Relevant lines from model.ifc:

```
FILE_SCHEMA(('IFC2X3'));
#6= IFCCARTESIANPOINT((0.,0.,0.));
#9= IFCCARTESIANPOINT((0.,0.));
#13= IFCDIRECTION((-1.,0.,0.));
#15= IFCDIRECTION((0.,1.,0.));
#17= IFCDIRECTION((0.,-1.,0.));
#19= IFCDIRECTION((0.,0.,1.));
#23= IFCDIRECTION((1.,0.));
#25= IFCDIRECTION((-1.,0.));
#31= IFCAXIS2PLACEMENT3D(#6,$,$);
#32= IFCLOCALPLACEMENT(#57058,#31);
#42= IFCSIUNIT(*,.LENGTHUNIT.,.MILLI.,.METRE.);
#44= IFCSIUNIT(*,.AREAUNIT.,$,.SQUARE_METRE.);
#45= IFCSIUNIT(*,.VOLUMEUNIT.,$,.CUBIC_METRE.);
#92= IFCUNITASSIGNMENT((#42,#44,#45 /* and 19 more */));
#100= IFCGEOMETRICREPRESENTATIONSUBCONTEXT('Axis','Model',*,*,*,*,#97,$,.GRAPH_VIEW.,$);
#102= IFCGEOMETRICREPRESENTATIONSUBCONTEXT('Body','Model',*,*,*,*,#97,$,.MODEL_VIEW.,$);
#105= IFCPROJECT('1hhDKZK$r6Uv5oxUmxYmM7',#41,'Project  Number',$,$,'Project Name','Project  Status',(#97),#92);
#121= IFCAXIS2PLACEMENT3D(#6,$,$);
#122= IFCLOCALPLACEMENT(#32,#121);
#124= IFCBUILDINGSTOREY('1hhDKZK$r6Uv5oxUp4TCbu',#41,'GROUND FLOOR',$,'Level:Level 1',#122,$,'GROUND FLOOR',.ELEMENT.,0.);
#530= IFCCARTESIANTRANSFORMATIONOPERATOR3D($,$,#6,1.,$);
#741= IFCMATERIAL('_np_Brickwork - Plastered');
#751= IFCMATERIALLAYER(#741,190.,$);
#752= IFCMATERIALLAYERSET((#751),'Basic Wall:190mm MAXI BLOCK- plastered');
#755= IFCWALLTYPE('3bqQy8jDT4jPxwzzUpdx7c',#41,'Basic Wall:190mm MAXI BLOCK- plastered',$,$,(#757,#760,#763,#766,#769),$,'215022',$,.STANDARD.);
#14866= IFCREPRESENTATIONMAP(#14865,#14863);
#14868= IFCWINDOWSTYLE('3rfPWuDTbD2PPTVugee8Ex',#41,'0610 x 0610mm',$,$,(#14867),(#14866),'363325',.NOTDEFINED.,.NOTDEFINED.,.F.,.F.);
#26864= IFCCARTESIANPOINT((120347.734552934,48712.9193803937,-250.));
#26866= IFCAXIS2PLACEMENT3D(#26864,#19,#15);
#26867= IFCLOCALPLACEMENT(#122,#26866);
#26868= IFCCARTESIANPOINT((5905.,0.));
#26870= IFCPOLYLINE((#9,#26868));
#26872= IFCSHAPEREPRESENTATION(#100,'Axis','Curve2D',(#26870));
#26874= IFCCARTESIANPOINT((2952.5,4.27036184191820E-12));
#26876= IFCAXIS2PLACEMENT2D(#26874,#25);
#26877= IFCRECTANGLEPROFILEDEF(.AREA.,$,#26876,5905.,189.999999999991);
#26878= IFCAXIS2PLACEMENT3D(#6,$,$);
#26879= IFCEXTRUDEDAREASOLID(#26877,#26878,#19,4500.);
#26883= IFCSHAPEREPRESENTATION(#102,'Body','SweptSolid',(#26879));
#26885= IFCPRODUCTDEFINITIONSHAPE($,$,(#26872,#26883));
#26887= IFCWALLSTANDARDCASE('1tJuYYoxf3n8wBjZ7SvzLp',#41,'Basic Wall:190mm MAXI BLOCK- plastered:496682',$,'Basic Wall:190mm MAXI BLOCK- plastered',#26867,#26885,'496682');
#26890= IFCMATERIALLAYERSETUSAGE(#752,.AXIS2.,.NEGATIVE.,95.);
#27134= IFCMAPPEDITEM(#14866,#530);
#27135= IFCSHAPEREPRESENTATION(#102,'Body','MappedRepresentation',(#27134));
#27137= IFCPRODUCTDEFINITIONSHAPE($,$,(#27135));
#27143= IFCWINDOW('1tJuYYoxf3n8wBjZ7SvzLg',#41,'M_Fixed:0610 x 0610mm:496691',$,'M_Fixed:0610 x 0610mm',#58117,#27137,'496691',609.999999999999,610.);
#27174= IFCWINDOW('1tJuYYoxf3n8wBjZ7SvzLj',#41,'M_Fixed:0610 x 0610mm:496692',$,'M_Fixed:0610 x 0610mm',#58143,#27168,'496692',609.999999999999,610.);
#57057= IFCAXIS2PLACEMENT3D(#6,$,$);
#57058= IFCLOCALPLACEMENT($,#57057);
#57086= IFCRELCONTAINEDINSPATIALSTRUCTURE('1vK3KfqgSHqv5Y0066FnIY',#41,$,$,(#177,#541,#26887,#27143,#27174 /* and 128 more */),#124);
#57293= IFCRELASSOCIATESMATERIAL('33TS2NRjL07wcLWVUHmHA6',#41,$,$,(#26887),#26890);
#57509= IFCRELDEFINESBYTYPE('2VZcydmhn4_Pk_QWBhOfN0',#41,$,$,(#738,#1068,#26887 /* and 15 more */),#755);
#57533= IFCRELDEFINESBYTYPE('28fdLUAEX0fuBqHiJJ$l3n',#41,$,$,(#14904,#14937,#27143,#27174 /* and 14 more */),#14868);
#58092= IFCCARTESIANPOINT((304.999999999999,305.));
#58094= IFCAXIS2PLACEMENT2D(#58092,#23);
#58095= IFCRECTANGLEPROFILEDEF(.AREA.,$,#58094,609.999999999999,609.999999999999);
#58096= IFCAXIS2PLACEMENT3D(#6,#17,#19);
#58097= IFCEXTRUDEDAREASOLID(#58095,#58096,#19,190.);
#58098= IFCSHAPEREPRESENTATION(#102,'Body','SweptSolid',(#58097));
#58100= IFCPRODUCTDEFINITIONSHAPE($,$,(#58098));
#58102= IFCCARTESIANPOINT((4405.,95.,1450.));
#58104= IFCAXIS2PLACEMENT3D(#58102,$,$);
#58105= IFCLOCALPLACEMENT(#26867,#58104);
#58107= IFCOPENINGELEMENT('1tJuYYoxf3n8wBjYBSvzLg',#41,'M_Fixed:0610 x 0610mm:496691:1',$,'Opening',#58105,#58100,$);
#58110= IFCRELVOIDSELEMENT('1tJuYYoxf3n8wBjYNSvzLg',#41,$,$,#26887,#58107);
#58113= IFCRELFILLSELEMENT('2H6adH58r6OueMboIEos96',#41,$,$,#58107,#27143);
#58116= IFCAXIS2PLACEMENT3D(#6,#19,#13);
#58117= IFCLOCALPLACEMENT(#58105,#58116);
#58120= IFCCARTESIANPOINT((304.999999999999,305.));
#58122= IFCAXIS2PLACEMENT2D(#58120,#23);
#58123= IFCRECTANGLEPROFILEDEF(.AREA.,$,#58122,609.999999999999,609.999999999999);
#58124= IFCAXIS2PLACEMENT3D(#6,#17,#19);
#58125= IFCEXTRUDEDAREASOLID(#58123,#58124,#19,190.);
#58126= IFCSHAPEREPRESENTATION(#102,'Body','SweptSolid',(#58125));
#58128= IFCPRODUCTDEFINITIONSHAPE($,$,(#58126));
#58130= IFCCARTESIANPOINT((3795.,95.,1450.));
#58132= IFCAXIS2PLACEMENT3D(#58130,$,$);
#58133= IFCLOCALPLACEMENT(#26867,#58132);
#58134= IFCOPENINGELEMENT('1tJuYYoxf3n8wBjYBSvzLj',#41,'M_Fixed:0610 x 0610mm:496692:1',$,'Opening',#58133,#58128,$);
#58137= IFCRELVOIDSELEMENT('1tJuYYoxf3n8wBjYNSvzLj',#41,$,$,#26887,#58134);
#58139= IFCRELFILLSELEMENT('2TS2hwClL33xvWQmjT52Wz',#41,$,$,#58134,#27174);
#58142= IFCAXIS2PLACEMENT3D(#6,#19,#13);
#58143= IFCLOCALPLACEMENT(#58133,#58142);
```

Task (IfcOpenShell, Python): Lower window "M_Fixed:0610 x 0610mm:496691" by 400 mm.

```python
import numpy as np
import ifcopenshell
import ifcopenshell.api.geometry
import ifcopenshell.util.placement
import ifcopenshell.util.unit

model = ifcopenshell.open("model.ifc")
unit_scale = ifcopenshell.util.unit.calculate_unit_scale(model)

window = model.by_id(27143)
opening = window.FillsVoids[0].RelatingOpeningElement
dz = -400.0

shift = np.array([0.0, 0.0, dz])
# The window is placed relative to its opening, so it follows when the opening moves.
matrix = ifcopenshell.util.placement.get_local_placement(opening.ObjectPlacement)
matrix[:3, 3] += shift
ifcopenshell.api.geometry.edit_object_placement(
    model, product=opening, matrix=matrix, is_si=False, should_transform_children=True
)

print(f"moved by {dz * unit_scale:+.3f} m")

model.write("model_edited.ifc")
```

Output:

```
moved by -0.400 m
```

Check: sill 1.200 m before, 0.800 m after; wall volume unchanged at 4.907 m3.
